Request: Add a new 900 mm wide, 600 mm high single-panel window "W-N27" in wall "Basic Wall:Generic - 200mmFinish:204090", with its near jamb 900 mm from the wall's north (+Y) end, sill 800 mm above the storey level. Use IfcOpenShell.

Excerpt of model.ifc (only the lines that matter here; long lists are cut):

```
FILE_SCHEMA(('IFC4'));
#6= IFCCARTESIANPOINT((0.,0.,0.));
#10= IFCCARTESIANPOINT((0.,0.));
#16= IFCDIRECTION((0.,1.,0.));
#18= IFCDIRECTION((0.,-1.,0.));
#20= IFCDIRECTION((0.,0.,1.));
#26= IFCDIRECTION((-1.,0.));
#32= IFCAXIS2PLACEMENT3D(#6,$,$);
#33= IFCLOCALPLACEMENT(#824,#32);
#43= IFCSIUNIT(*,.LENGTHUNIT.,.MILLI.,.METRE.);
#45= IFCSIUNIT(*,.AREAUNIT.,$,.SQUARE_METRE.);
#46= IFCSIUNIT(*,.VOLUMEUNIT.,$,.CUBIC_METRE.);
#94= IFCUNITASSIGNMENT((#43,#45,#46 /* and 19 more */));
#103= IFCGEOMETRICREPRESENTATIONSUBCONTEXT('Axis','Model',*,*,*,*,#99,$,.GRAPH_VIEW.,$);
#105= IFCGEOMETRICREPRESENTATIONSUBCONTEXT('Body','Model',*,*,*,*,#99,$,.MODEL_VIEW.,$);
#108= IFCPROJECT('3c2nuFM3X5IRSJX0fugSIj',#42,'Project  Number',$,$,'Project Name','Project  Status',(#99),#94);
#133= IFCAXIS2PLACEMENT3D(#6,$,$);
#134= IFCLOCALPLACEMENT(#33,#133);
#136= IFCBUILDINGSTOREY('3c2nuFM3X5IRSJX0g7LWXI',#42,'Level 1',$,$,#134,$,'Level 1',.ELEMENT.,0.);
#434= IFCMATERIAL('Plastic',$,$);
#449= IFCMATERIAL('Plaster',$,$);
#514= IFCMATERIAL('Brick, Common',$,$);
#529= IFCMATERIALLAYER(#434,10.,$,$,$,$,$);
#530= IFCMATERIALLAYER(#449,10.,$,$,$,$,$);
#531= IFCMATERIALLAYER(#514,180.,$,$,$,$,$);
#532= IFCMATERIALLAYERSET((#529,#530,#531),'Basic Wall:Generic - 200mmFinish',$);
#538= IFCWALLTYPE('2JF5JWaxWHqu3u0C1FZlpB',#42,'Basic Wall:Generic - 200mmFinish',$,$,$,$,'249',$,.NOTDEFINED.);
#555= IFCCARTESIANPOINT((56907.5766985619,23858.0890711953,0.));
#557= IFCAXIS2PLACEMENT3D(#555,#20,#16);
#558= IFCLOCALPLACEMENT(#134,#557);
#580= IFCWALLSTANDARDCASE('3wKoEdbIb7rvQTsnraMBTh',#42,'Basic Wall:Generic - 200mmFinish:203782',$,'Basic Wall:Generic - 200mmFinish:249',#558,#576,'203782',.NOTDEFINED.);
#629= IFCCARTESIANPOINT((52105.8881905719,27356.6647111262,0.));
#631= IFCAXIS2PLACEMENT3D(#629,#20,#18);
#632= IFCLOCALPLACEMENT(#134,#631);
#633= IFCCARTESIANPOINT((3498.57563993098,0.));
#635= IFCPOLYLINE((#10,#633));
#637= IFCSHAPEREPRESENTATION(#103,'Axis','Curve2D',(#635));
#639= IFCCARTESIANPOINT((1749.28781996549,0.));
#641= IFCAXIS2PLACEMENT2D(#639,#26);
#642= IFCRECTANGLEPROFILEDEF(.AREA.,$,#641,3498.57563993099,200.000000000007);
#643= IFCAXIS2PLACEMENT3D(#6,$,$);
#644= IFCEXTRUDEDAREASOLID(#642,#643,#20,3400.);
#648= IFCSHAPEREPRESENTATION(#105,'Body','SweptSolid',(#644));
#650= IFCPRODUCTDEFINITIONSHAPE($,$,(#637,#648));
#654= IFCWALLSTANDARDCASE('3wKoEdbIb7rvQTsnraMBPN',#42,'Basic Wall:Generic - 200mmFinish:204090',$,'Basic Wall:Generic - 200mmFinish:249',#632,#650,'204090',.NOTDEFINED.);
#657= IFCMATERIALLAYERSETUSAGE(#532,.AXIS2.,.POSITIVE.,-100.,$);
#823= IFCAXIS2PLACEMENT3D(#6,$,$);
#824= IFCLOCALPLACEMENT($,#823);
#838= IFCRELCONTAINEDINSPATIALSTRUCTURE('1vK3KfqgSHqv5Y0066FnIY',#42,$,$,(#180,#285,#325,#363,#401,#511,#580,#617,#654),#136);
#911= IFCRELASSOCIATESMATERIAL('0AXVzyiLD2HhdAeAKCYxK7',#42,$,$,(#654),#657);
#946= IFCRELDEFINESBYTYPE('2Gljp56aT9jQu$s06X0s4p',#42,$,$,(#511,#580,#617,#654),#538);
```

```python
import numpy as np
import ifcopenshell
import ifcopenshell.api.feature
import ifcopenshell.api.geometry
import ifcopenshell.api.root
import ifcopenshell.api.spatial
import ifcopenshell.geom
import ifcopenshell.util.element
import ifcopenshell.util.placement
import ifcopenshell.util.representation
import ifcopenshell.util.shape
import ifcopenshell.util.unit

model = ifcopenshell.open("model.ifc")
unit_scale = ifcopenshell.util.unit.calculate_unit_scale(model)
settings = ifcopenshell.geom.settings()


def volume(element):
    """Net volume in cubic metres, openings subtracted."""
    shape = ifcopenshell.geom.create_shape(settings, element)
    return ifcopenshell.util.shape.get_volume(shape.geometry)


wall = model.by_guid("3wKoEdbIb7rvQTsnraMBPN")
storey = ifcopenshell.util.element.get_container(wall, ifc_class="IfcBuildingStorey")
context = ifcopenshell.util.representation.get_context(model, "Model", "Body", "MODEL_VIEW")
before = volume(wall)

width, height, from_end, sill = 0.9, 0.6, 0.9, 0.8  # metres

# The wall runs along its own X axis, and the end named is its -X end.
wall_shape = ifcopenshell.geom.create_shape(settings, wall)
x, y, z = ifcopenshell.util.shape.get_vertices(wall_shape.geometry).T
start = x.min() + from_end
face, thickness = float(y.min()), float(y.max() - y.min())
wall_matrix = ifcopenshell.util.placement.get_local_placement(wall.ObjectPlacement)
level = ifcopenshell.util.placement.get_local_placement(storey.ObjectPlacement)[2, 3]


def in_wall(x, y):
    """Placement at x, y metres in the wall's axes, at sill height."""
    matrix = wall_matrix.copy()
    matrix[:, 3] = wall_matrix @ np.array([x / unit_scale, y / unit_scale, 0.0, 1.0])
    matrix[2, 3] = level + sill / unit_scale
    return matrix


# Opening: a box that overshoots both wall faces by 50 mm.
opening = ifcopenshell.api.root.create_entity(model, ifc_class="IfcOpeningElement", predefined_type="OPENING")
box = ifcopenshell.api.geometry.add_wall_representation(
    model, context=context, length=width, height=height, thickness=thickness + 0.1
)
ifcopenshell.api.geometry.assign_representation(model, product=opening, representation=box)
ifcopenshell.api.geometry.edit_object_placement(model, product=opening, matrix=in_wall(start, face - 0.05), is_si=False)
ifcopenshell.api.feature.add_feature(model, feature=opening, element=wall)

window = ifcopenshell.api.root.create_entity(model, ifc_class="IfcWindow", name="W-N27", predefined_type="WINDOW")
window.OverallWidth, window.OverallHeight = width / unit_scale, height / unit_scale
window.PartitioningType = "SINGLE_PANEL"
body = ifcopenshell.api.geometry.add_window_representation(
    model,
    context=context,
    overall_width=window.OverallWidth,
    overall_height=window.OverallHeight,
    partition_type="SINGLE_PANEL",
)
ifcopenshell.api.geometry.assign_representation(model, product=window, representation=body)
ifcopenshell.api.spatial.assign_container(model, products=[window], relating_structure=storey)
ifcopenshell.api.feature.add_filling(model, opening=opening, element=window)

# Centre the window in the wall's thickness.
ifcopenshell.api.geometry.edit_object_placement(model, product=window, matrix=in_wall(start, face), is_si=False)
window_shape = ifcopenshell.geom.create_shape(settings, window)
depth = ifcopenshell.util.shape.get_vertices(window_shape.geometry)[:, 1]
offset = face + thickness / 2 - (depth.min() + depth.max()) / 2
ifcopenshell.api.geometry.edit_object_placement(model, product=window, matrix=in_wall(start, offset), is_si=False)

after = volume(wall)

print(f"wall volume {before:.3f} -> {after:.3f} m3")

model.write("model-out.ifc")
```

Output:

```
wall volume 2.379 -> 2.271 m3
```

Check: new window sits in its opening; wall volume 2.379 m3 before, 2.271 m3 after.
